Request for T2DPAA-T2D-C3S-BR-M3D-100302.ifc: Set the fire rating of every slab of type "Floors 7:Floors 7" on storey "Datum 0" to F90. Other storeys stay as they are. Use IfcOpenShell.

First a look at what the model holds.

```python
import ifcopenshell
import ifcopenshell.util.element

model = ifcopenshell.open("T2DPAA-T2D-C3S-BR-M3D-100302.ifc")
print(model.schema)
storey = next(s for s in model.by_type("IfcBuildingStorey") if s.Name == "Datum 0")
slabs = [e for e in ifcopenshell.util.element.get_decomposition(storey) if e.is_a("IfcSlab")]
seen = {}
for e in slabs:
    element_type = ifcopenshell.util.element.get_type(e)
    key = (element_type.Name if element_type != e and element_type else None, ifcopenshell.util.element.get_pset(e, "Pset_SlabCommon", "FireRating"))
    seen[key] = seen.get(key, 0) + 1
for (name, value), count in sorted(seen.items(), key=str):
    print(count, "x", name, "|", value)
```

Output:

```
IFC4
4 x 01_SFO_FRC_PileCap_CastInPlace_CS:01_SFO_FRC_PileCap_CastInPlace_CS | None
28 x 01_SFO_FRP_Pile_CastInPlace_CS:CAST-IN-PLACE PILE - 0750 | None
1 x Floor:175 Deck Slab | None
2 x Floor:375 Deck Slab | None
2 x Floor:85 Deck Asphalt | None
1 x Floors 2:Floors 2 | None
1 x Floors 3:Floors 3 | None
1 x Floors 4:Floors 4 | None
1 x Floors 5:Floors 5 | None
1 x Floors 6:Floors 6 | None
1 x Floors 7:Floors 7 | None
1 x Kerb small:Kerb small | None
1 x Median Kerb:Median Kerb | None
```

```python
import ifcopenshell
import ifcopenshell.api.pset
import ifcopenshell.util.element

model = ifcopenshell.open("T2DPAA-T2D-C3S-BR-M3D-100302.ifc")

storey = next(s for s in model.by_type("IfcBuildingStorey") if s.Name == "Datum 0")
slabs = [e for e in ifcopenshell.util.element.get_decomposition(storey) if e.is_a("IfcSlab")]

count = 0
for e in slabs:
    element_type = ifcopenshell.util.element.get_type(e)
    if element_type in (None, e) or element_type.Name != "Floors 7:Floors 7":
        continue
    # add_pset returns the element's existing set when there is one.
    pset = ifcopenshell.api.pset.add_pset(model, product=e, name="Pset_SlabCommon")
    ifcopenshell.api.pset.edit_pset(model, pset=pset, properties={"FireRating": "F90"})
    count += 1

print(count, "slabs updated")

model.write("T2DPAA-T2D-C3S-BR-M3D-100302_v2.ifc")
```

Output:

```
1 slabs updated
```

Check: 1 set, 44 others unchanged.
